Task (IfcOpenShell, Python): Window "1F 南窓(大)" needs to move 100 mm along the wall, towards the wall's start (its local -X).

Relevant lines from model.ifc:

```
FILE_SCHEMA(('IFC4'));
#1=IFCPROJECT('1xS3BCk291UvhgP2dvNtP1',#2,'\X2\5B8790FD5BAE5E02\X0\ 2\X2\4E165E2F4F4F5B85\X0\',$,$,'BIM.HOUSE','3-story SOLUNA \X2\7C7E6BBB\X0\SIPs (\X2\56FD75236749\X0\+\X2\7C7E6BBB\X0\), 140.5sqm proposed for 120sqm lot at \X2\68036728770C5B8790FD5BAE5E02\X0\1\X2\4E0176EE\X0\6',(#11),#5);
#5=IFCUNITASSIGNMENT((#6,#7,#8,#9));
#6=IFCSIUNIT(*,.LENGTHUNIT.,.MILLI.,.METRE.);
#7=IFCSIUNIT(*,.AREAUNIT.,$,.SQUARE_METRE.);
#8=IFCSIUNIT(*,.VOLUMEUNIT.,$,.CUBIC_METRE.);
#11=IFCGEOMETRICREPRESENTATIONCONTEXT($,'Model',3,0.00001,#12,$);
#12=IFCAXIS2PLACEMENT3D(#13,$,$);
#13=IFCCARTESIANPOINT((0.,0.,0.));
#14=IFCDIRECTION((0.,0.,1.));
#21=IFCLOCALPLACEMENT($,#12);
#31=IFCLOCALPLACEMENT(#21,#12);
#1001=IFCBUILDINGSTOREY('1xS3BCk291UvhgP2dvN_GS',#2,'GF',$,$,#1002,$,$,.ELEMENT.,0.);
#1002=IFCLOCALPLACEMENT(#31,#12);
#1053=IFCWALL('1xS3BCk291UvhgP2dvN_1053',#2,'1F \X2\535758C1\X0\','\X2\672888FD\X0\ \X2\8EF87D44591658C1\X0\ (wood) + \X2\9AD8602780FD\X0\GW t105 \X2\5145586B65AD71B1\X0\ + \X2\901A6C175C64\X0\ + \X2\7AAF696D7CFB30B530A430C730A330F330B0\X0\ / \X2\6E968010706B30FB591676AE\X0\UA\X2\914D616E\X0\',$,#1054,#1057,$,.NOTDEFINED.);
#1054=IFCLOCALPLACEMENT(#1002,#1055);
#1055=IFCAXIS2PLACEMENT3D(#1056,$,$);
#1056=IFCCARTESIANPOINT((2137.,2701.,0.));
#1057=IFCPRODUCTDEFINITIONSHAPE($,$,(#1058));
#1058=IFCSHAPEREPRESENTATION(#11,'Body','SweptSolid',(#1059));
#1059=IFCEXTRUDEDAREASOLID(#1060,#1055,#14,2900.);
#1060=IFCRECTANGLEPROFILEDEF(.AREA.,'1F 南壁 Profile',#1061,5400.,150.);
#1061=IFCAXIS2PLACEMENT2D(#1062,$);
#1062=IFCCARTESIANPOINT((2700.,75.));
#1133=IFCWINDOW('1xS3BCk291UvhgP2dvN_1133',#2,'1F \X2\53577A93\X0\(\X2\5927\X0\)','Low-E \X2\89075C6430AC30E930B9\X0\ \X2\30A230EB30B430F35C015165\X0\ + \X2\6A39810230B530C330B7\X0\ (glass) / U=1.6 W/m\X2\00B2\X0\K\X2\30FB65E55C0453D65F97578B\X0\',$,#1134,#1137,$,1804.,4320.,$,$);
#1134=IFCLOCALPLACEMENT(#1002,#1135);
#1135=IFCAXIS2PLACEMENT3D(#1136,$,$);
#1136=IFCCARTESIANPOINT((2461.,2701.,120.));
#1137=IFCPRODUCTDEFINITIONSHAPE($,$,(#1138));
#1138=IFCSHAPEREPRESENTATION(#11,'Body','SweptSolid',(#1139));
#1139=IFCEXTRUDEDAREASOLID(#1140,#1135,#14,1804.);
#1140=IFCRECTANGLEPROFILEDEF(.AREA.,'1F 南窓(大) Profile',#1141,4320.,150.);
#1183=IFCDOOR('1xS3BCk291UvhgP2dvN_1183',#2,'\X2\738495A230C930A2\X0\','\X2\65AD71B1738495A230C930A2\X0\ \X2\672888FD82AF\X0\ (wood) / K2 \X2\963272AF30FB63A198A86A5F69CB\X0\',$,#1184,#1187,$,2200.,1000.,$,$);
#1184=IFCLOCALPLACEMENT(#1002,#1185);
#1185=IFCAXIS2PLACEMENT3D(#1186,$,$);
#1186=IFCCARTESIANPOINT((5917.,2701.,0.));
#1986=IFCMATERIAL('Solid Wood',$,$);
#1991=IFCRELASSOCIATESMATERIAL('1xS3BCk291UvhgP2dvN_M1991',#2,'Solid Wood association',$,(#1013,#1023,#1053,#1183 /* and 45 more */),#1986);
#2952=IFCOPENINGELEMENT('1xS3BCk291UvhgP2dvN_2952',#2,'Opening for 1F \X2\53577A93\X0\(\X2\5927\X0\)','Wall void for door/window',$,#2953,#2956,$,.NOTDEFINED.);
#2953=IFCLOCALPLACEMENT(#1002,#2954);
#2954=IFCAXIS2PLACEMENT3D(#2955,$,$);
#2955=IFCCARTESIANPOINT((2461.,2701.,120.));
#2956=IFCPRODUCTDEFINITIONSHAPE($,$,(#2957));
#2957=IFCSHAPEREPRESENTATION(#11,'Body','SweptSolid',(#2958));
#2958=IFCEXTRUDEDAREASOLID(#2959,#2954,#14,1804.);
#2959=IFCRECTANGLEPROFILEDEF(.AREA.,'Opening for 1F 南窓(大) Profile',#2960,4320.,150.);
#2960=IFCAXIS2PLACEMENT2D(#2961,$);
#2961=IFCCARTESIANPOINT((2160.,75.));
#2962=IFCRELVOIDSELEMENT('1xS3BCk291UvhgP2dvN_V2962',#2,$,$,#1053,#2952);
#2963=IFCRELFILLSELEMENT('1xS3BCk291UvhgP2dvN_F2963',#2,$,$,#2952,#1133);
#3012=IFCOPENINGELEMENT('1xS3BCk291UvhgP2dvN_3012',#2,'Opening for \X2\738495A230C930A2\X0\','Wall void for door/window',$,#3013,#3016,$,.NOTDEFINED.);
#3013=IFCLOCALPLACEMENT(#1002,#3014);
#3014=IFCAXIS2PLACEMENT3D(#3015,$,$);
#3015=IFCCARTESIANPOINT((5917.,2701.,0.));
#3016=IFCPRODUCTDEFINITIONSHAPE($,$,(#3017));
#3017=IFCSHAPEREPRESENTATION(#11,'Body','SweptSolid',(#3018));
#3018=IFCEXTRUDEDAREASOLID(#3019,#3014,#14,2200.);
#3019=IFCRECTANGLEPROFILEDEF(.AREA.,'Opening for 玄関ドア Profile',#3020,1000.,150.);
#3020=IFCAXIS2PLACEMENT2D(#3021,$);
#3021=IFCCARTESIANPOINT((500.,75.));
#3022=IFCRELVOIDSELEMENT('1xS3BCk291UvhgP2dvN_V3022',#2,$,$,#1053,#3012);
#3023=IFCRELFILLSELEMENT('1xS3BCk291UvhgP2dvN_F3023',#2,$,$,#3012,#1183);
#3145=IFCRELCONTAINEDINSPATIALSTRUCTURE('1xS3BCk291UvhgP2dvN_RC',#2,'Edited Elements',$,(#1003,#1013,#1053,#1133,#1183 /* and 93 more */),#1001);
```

```python
import ifcopenshell
import ifcopenshell.api.geometry
import ifcopenshell.util.placement

model = ifcopenshell.open("model.ifc")

window = model.by_guid("1xS3BCk291UvhgP2dvN_1133")
opening = window.FillsVoids[0].RelatingOpeningElement
wall = opening.VoidsElements[0].RelatingBuildingElement

wall_matrix = ifcopenshell.util.placement.get_local_placement(wall.ObjectPlacement)
shift = wall_matrix[:3, 0] * -100.0
before = ifcopenshell.util.placement.get_local_placement(window.ObjectPlacement)[:3, 3].copy()

# The window is not placed relative to its opening, so move both.
for product in (opening, window):
    matrix = ifcopenshell.util.placement.get_local_placement(product.ObjectPlacement)
    matrix[:3, 3] += shift
    ifcopenshell.api.geometry.edit_object_placement(model, product=product, matrix=matrix, is_si=False)

after = ifcopenshell.util.placement.get_local_placement(window.ObjectPlacement)[:3, 3]
print("window moved by", (after - before).round(3) + 0.0)

model.write("model_updated.ifc")
```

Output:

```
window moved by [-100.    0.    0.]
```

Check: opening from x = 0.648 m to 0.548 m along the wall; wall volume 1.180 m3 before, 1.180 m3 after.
